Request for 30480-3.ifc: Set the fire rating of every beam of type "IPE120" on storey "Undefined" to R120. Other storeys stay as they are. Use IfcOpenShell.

First a look at what the model holds.

```python
import ifcopenshell
import ifcopenshell.util.element

model = ifcopenshell.open("30480-3.ifc")
print(model.schema)
storey = next(s for s in model.by_type("IfcBuildingStorey") if s.Name == "Undefined")
beams = [e for e in ifcopenshell.util.element.get_decomposition(storey) if e.is_a("IfcBeam")]
seen = {}
for e in beams:
    element_type = ifcopenshell.util.element.get_type(e)
    key = (element_type.Name if element_type != e and element_type else None, ifcopenshell.util.element.get_pset(e, "Pset_BeamCommon", "FireRating"))
    seen[key] = seen.get(key, 0) + 1
for (name, value), count in sorted(seen.items(), key=str):
    print(count, "x", name, "|", value)
```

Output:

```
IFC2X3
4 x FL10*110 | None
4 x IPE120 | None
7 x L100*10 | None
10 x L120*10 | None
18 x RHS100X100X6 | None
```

```python
import ifcopenshell
import ifcopenshell.api.pset
import ifcopenshell.util.element

model = ifcopenshell.open("30480-3.ifc")

storey = next(s for s in model.by_type("IfcBuildingStorey") if s.Name == "Undefined")
beams = [e for e in ifcopenshell.util.element.get_decomposition(storey) if e.is_a("IfcBeam")]

count = 0
for e in beams:
    element_type = ifcopenshell.util.element.get_type(e)
    if element_type in (None, e) or element_type.Name != "IPE120":
        continue
    found = ifcopenshell.util.element.get_pset(e, "Pset_BeamCommon", should_inherit=False)
    if found:
        pset = model.by_id(found["id"])
        if len(ifcopenshell.util.element.get_elements_by_pset(pset)) > 1:
            pset = ifcopenshell.api.pset.unshare_pset(model, products=[e], pset=pset)[0]
    else:
        pset = ifcopenshell.api.pset.add_pset(model, product=e, name="Pset_BeamCommon")
    ifcopenshell.api.pset.edit_pset(model, pset=pset, properties={"FireRating": "R120"})
    count += 1

print(count, "beams updated")

model.write("30480-3_v2.ifc")
```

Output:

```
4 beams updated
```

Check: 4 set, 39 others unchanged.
